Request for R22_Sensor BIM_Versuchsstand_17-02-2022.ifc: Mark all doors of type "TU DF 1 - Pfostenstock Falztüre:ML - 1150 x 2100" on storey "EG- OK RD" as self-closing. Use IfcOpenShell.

First a look at what the model holds.

```python
import ifcopenshell
import ifcopenshell.util.element

model = ifcopenshell.open("R22_Sensor BIM_Versuchsstand_17-02-2022.ifc")
print(model.schema)
storey = next(s for s in model.by_type("IfcBuildingStorey") if s.Name == "EG- OK RD")
doors = [e for e in ifcopenshell.util.element.get_decomposition(storey) if e.is_a("IfcDoor")]
seen = {}
for e in doors:
    element_type = ifcopenshell.util.element.get_type(e)
    key = (element_type.Name if element_type != e and element_type else None, ifcopenshell.util.element.get_pset(e, "Pset_DoorCommon", "SelfClosing"))
    seen[key] = seen.get(key, 0) + 1
for (name, value), count in sorted(seen.items(), key=str):
    print(count, "x", name, "|", value)
```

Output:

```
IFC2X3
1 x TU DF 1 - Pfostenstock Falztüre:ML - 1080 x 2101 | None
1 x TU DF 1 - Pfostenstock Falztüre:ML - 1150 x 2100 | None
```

```python
import ifcopenshell
import ifcopenshell.api.pset
import ifcopenshell.util.element

model = ifcopenshell.open("R22_Sensor BIM_Versuchsstand_17-02-2022.ifc")

storey = next(s for s in model.by_type("IfcBuildingStorey") if s.Name == "EG- OK RD")
doors = [e for e in ifcopenshell.util.element.get_decomposition(storey) if e.is_a("IfcDoor")]

count = 0
for e in doors:
    element_type = ifcopenshell.util.element.get_type(e)
    if element_type in (None, e) or element_type.Name != "TU DF 1 - Pfostenstock Falztüre:ML - 1150 x 2100":
        continue
    # add_pset returns the element's existing set when there is one.
    pset = ifcopenshell.api.pset.add_pset(model, product=e, name="Pset_DoorCommon")
    ifcopenshell.api.pset.edit_pset(model, pset=pset, properties={"SelfClosing": True})
    count += 1

print(count, "doors updated")

model.write("R22_Sensor BIM_Versuchsstand_17-02-2022_v2.ifc")
```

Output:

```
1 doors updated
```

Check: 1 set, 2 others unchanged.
